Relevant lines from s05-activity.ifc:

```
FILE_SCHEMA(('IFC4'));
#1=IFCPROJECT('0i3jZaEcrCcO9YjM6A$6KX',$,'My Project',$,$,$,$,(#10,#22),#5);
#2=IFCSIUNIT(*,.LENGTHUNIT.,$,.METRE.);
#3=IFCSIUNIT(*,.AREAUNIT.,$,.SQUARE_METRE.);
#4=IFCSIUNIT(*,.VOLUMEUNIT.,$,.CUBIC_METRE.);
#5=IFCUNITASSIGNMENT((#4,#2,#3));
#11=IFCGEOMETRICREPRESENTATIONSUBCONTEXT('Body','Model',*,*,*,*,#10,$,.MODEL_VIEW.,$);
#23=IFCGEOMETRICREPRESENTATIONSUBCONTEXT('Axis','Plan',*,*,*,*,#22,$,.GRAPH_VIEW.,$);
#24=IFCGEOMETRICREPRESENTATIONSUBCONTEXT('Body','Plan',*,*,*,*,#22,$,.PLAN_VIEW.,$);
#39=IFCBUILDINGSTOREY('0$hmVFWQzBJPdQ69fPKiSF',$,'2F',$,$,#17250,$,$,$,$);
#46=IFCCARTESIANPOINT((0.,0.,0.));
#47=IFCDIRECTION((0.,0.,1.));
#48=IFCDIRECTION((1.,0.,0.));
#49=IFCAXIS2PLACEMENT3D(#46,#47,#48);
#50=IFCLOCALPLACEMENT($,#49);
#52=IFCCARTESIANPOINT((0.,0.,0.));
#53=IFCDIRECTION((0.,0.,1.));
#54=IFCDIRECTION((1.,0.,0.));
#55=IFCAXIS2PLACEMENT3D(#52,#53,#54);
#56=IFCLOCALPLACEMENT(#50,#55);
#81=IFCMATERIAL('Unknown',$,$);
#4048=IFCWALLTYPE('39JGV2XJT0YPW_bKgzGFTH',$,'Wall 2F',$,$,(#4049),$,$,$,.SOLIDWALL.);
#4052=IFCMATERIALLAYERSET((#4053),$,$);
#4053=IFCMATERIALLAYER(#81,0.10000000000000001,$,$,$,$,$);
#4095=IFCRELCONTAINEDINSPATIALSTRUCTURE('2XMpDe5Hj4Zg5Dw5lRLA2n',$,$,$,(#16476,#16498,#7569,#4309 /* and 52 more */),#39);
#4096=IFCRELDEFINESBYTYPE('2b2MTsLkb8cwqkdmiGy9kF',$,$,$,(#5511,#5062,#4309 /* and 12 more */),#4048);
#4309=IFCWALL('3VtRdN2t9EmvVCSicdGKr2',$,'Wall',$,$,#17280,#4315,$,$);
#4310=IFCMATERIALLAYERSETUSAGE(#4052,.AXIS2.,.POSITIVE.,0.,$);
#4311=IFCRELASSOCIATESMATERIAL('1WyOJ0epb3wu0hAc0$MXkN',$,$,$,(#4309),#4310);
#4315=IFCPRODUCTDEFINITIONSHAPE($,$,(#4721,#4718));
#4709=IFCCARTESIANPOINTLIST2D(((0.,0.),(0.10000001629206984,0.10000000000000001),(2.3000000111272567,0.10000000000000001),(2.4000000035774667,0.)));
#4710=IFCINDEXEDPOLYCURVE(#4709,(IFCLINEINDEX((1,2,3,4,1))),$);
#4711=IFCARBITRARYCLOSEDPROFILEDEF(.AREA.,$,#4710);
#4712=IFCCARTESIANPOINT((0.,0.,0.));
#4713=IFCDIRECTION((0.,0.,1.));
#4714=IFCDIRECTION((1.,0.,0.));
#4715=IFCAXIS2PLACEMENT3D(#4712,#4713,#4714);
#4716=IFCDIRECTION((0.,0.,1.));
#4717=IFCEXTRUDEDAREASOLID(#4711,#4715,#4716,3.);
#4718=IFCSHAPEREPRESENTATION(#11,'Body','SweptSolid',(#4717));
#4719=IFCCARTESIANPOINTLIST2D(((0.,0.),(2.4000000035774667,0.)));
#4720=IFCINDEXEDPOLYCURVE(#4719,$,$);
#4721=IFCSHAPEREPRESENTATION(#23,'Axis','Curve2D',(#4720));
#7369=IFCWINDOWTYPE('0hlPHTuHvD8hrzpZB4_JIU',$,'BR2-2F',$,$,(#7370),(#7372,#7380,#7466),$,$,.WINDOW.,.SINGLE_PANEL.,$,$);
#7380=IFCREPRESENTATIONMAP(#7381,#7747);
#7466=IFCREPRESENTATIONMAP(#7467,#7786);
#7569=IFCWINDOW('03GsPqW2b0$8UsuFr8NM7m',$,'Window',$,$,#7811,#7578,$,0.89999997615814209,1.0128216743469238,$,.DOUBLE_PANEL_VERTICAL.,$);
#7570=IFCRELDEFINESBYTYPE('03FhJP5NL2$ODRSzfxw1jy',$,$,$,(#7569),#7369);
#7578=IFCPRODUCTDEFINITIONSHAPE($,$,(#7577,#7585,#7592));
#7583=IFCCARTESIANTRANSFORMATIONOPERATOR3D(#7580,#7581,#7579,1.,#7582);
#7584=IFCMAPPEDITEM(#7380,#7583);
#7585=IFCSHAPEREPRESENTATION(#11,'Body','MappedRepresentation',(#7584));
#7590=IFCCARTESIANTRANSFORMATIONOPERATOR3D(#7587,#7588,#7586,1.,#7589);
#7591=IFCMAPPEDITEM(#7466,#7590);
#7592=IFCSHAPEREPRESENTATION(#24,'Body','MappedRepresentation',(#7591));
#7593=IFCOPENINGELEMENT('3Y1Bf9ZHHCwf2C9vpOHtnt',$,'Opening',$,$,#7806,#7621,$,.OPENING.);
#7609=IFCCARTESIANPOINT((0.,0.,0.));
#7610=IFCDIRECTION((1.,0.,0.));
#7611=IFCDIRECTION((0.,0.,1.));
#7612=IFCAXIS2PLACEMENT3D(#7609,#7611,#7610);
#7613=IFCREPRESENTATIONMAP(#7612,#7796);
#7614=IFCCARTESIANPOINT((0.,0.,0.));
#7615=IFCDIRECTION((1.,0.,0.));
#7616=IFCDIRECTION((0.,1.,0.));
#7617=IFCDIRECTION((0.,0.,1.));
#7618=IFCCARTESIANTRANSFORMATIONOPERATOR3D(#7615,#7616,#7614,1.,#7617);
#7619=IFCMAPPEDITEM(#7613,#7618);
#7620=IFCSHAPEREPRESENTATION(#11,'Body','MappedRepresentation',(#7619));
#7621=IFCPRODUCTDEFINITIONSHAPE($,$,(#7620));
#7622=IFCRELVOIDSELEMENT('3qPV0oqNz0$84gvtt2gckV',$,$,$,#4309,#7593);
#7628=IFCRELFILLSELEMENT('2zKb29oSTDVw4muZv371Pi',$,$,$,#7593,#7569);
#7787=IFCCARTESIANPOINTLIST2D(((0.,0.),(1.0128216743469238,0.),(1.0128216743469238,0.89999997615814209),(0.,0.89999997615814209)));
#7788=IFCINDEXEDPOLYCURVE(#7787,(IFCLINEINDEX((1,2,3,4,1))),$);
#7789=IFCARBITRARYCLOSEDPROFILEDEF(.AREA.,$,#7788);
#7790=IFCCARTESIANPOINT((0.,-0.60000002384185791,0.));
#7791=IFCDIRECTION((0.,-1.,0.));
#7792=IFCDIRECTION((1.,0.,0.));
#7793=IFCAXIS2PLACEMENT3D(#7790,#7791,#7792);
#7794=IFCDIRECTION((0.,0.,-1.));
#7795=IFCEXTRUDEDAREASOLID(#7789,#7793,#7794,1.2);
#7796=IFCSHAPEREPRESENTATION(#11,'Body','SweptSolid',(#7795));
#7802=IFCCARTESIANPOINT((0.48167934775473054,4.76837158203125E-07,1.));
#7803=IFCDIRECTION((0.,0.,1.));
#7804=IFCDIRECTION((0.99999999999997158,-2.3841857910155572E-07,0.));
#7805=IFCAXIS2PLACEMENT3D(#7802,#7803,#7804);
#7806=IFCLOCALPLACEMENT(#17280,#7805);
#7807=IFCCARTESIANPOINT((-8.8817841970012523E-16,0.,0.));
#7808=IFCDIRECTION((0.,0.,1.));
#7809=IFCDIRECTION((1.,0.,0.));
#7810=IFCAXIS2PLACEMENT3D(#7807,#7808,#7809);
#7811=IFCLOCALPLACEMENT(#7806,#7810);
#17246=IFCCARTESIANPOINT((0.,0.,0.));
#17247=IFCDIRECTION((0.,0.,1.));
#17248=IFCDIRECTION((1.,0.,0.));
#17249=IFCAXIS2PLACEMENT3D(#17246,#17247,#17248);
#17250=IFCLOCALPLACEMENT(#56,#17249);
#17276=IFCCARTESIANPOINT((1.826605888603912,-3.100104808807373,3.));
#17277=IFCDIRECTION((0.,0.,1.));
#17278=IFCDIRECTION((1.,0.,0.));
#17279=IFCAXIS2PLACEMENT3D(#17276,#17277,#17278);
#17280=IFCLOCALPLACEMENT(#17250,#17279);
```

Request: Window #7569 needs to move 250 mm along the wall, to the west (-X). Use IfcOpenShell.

```python
import ifcopenshell
import ifcopenshell.api.geometry
import ifcopenshell.util.placement
import ifcopenshell.util.unit

model = ifcopenshell.open("s05-activity.ifc")
unit_scale = ifcopenshell.util.unit.calculate_unit_scale(model)

window = model.by_id(7569)
opening = window.FillsVoids[0].RelatingOpeningElement
wall = opening.VoidsElements[0].RelatingBuildingElement

wall_matrix = ifcopenshell.util.placement.get_local_placement(wall.ObjectPlacement)
shift = wall_matrix[:3, 0] * -0.25 / unit_scale
before = ifcopenshell.util.placement.get_local_placement(window.ObjectPlacement)[:3, 3].copy()

# The window is placed relative to its opening, so it follows when the opening moves.
matrix = ifcopenshell.util.placement.get_local_placement(opening.ObjectPlacement)
matrix[:3, 3] += shift
ifcopenshell.api.geometry.edit_object_placement(
    model, product=opening, matrix=matrix, is_si=False, should_transform_children=True
)

after = ifcopenshell.util.placement.get_local_placement(window.ObjectPlacement)[:3, 3]
print("window moved by", (after - before).round(3) + 0.0)

model.write("s05-activity-out.ifc")
```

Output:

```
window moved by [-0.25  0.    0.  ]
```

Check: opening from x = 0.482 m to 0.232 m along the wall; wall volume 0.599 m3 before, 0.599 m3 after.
